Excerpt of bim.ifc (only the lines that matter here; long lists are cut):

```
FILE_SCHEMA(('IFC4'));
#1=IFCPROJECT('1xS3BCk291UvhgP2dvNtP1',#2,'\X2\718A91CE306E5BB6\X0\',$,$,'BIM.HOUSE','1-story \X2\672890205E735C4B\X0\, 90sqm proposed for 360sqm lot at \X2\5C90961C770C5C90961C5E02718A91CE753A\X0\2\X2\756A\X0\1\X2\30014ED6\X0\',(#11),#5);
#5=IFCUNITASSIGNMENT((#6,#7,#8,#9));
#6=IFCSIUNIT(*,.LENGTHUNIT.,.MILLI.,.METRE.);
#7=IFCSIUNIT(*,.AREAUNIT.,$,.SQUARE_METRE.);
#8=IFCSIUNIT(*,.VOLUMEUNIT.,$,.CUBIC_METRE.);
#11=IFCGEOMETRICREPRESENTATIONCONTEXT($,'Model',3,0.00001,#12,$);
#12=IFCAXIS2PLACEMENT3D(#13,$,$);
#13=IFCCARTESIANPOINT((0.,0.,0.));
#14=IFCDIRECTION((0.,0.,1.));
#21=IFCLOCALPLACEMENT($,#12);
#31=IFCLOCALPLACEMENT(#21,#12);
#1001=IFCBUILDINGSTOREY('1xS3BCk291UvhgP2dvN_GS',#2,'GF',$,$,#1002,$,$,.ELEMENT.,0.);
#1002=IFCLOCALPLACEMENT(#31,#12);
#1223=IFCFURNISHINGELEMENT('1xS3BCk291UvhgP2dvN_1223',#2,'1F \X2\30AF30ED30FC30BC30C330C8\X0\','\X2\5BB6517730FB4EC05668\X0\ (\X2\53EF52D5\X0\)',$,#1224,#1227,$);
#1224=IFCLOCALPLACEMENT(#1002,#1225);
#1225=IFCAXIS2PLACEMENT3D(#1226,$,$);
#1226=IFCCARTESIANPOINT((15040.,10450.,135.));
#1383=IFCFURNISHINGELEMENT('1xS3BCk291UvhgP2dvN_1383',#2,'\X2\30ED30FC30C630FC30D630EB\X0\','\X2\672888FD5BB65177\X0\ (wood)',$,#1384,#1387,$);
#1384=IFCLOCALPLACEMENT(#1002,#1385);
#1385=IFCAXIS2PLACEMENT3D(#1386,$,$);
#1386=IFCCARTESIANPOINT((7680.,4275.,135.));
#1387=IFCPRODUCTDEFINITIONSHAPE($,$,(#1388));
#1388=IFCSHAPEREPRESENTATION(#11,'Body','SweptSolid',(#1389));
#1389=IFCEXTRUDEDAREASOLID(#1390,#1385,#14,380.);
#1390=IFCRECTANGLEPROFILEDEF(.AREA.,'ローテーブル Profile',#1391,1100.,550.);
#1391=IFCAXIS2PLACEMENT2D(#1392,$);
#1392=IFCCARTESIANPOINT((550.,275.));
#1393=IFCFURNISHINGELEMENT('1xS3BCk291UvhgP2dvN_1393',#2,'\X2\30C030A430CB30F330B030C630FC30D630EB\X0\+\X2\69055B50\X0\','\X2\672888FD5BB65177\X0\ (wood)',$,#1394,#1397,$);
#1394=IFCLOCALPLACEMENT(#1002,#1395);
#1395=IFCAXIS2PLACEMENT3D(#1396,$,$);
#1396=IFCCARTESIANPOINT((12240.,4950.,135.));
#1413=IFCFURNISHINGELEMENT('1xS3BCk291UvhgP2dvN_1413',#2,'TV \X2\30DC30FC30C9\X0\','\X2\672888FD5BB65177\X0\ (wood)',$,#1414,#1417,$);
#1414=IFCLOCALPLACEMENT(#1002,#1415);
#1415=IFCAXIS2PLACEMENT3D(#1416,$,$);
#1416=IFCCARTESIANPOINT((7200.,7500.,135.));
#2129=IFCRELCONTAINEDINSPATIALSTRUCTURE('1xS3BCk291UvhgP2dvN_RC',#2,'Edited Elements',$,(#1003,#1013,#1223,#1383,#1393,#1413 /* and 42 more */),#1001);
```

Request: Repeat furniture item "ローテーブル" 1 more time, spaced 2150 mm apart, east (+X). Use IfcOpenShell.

```python
import numpy as np
import ifcopenshell
import ifcopenshell.api.geometry
import ifcopenshell.api.root
import ifcopenshell.util.element
import ifcopenshell.util.placement
import ifcopenshell.util.unit

model = ifcopenshell.open("bim.ifc")
unit_scale = ifcopenshell.util.unit.calculate_unit_scale(model)


def reuse_history(source, copy):
    """copy_class also copies each property set's owner history, people and application; keep the originals."""
    for rel in copy.IsDefinedBy:
        if rel.is_a("IfcRelDefinesByProperties") and (history := rel.RelatingPropertyDefinition.OwnerHistory):
            rel.RelatingPropertyDefinition.OwnerHistory = source.OwnerHistory
            ifcopenshell.util.element.remove_deep2(model, history)


source = model.by_guid("1xS3BCk291UvhgP2dvN_1383")
base = ifcopenshell.util.placement.get_local_placement(source.ObjectPlacement)
step = np.array([1.0, 0.0, 0.0]) * 2.15 / unit_scale

for i in range(1, 2):
    copy = ifcopenshell.api.root.copy_class(model, product=source)
    copy.Representation = ifcopenshell.util.element.copy_deep(
        model, source.Representation, exclude=["IfcGeometricRepresentationContext", "IfcRepresentationMap"]
    )
    reuse_history(source, copy)
    matrix = base.copy()
    matrix[:3, 3] += i * step
    print("added at", matrix[:3, 3].round(3) + 0.0)
    ifcopenshell.api.geometry.edit_object_placement(model, product=copy, matrix=matrix, is_si=False)

model.write("bim_updated.ifc")
```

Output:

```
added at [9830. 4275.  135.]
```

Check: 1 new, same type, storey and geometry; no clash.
